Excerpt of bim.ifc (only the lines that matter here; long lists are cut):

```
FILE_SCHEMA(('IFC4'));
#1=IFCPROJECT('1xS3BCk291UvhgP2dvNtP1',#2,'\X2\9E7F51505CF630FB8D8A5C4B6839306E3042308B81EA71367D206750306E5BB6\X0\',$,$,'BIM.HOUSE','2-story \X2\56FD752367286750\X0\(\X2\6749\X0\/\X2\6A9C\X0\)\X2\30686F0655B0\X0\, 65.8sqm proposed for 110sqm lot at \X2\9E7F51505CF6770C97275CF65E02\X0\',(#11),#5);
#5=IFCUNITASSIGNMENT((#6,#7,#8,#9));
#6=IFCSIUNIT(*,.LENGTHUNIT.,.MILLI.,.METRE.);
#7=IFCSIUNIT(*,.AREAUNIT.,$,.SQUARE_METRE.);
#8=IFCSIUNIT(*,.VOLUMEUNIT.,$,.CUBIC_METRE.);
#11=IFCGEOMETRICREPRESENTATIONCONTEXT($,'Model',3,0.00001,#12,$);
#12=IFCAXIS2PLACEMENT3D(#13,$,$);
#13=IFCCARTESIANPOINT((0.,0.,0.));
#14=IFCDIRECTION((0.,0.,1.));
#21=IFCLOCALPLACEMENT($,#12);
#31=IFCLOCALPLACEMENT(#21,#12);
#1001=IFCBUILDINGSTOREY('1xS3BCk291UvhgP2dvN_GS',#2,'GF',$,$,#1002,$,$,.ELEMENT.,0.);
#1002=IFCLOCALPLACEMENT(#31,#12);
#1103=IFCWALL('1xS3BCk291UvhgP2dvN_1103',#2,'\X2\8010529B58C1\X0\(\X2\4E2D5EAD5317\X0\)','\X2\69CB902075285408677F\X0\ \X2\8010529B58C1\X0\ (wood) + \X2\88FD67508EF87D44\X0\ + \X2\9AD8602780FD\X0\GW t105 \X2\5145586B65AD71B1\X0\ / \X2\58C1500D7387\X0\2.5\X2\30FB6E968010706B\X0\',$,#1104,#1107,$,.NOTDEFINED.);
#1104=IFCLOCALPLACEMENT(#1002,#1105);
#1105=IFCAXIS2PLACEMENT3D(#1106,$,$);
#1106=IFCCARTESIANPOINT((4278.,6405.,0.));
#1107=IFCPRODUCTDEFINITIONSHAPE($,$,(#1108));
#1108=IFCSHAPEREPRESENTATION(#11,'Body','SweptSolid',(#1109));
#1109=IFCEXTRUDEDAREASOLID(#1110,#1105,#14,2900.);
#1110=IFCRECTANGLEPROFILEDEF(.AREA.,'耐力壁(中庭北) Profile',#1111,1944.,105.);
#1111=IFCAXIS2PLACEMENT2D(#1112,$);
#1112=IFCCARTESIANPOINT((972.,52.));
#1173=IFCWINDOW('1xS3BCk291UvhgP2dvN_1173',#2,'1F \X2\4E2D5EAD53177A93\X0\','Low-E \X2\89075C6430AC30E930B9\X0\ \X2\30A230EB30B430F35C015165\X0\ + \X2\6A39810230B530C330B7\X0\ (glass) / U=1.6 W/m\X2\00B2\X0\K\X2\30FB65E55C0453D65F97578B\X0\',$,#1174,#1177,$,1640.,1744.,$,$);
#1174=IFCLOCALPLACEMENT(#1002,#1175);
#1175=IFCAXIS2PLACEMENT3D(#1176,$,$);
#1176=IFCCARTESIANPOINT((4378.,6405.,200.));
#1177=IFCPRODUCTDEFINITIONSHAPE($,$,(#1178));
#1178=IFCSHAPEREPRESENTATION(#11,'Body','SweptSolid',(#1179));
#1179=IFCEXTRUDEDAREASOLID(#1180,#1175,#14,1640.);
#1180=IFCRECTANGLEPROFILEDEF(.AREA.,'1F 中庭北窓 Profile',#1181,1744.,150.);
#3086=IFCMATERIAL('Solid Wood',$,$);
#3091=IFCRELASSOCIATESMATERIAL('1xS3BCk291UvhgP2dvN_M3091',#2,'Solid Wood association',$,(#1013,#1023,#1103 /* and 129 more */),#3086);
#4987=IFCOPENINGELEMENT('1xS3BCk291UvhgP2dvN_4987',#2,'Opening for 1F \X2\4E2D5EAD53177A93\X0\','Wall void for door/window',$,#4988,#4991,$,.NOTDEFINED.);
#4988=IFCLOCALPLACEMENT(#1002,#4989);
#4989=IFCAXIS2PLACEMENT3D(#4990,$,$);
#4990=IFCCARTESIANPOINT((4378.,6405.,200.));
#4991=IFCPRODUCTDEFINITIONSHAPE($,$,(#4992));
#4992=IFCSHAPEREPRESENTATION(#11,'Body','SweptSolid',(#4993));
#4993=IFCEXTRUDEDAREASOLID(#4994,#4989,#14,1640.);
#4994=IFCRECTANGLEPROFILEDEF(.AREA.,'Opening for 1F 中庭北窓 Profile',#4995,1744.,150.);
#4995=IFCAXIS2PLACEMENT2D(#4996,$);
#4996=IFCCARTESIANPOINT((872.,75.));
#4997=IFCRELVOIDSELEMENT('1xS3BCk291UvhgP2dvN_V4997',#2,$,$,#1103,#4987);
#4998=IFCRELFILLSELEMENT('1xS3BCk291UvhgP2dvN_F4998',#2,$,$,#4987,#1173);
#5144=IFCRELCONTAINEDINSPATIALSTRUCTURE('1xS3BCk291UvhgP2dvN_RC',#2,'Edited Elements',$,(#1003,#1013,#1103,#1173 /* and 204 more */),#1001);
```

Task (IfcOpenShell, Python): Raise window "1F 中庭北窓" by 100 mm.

```python
import numpy as np
import ifcopenshell
import ifcopenshell.api.geometry
import ifcopenshell.util.placement
import ifcopenshell.util.unit

model = ifcopenshell.open("bim.ifc")
unit_scale = ifcopenshell.util.unit.calculate_unit_scale(model)

window = model.by_guid("1xS3BCk291UvhgP2dvN_1173")
opening = window.FillsVoids[0].RelatingOpeningElement
dz = 0.1 / unit_scale

shift = np.array([0.0, 0.0, dz])
# The window is not placed relative to its opening, so move both.
for product in (opening, window):
    matrix = ifcopenshell.util.placement.get_local_placement(product.ObjectPlacement)
    matrix[:3, 3] += shift
    ifcopenshell.api.geometry.edit_object_placement(model, product=product, matrix=matrix, is_si=False)

print(f"moved by {dz * unit_scale:+.3f} m")

model.write("bim-out.ifc")
```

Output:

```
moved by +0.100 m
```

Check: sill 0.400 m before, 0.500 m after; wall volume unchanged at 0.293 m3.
